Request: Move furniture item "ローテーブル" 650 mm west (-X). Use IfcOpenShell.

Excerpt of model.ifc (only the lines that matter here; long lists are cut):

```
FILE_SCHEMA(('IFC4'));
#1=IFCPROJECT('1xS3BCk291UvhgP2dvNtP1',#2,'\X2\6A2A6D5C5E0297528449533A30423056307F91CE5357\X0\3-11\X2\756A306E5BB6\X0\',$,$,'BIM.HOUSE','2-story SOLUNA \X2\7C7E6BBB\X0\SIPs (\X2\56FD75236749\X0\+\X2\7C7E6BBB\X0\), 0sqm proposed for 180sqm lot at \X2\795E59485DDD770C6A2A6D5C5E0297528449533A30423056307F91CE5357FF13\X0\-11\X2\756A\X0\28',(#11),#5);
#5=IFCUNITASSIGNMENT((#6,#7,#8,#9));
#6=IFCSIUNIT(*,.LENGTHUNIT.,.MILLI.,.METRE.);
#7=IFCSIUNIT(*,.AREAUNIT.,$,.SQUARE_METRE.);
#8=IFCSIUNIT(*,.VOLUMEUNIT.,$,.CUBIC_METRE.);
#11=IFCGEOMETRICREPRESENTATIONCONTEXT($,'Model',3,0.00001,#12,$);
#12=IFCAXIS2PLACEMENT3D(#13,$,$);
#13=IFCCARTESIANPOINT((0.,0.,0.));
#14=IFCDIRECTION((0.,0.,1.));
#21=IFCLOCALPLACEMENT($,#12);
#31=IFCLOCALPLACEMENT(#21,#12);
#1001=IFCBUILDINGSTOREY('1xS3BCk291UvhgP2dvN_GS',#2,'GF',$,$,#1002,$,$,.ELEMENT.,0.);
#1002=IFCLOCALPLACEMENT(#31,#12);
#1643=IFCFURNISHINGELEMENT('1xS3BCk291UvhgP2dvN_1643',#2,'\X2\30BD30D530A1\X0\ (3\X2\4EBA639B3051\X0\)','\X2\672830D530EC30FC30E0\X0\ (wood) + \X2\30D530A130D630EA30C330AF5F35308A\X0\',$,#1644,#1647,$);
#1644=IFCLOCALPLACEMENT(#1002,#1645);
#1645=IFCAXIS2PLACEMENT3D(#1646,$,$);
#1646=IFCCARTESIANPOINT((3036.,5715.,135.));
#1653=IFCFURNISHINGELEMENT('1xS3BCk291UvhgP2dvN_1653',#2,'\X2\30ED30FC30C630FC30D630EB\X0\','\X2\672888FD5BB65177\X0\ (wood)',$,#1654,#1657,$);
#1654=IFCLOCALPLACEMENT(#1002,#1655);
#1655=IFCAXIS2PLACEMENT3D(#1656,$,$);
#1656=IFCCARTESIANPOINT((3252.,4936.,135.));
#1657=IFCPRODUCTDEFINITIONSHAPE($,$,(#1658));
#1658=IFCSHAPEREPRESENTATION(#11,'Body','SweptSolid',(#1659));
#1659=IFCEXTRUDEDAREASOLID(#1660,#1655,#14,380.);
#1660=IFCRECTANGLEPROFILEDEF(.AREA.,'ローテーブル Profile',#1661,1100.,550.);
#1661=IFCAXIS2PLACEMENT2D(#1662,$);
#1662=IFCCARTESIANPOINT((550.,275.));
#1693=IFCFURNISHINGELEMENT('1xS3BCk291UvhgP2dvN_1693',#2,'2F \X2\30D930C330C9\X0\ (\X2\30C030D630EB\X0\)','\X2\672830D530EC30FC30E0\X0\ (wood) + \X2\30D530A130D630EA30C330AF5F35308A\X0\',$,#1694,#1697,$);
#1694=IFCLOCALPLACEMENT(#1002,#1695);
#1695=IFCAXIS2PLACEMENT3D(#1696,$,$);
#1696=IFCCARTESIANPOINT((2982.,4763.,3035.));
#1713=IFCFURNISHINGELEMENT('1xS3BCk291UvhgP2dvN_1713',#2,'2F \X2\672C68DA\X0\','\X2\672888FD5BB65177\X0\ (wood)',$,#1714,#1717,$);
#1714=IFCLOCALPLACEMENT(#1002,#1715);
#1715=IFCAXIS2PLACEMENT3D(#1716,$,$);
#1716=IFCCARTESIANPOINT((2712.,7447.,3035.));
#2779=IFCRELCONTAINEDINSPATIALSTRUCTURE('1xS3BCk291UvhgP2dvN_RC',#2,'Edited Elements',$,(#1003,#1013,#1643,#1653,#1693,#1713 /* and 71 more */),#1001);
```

```python
import ifcopenshell
import ifcopenshell.api.geometry
import ifcopenshell.util.placement

model = ifcopenshell.open("model.ifc")

item = model.by_guid("1xS3BCk291UvhgP2dvN_1653")
matrix = ifcopenshell.util.placement.get_local_placement(item.ObjectPlacement)
matrix[0, 3] -= 650.0
ifcopenshell.api.geometry.edit_object_placement(model, product=item, matrix=matrix, is_si=False)

print(ifcopenshell.util.placement.get_local_placement(item.ObjectPlacement).round(3) + 0.0)

model.write("model_rev.ifc")
```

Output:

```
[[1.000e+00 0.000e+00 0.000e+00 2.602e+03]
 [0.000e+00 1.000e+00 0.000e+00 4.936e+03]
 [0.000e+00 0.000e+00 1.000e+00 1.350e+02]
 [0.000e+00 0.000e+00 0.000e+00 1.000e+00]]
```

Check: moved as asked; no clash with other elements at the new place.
